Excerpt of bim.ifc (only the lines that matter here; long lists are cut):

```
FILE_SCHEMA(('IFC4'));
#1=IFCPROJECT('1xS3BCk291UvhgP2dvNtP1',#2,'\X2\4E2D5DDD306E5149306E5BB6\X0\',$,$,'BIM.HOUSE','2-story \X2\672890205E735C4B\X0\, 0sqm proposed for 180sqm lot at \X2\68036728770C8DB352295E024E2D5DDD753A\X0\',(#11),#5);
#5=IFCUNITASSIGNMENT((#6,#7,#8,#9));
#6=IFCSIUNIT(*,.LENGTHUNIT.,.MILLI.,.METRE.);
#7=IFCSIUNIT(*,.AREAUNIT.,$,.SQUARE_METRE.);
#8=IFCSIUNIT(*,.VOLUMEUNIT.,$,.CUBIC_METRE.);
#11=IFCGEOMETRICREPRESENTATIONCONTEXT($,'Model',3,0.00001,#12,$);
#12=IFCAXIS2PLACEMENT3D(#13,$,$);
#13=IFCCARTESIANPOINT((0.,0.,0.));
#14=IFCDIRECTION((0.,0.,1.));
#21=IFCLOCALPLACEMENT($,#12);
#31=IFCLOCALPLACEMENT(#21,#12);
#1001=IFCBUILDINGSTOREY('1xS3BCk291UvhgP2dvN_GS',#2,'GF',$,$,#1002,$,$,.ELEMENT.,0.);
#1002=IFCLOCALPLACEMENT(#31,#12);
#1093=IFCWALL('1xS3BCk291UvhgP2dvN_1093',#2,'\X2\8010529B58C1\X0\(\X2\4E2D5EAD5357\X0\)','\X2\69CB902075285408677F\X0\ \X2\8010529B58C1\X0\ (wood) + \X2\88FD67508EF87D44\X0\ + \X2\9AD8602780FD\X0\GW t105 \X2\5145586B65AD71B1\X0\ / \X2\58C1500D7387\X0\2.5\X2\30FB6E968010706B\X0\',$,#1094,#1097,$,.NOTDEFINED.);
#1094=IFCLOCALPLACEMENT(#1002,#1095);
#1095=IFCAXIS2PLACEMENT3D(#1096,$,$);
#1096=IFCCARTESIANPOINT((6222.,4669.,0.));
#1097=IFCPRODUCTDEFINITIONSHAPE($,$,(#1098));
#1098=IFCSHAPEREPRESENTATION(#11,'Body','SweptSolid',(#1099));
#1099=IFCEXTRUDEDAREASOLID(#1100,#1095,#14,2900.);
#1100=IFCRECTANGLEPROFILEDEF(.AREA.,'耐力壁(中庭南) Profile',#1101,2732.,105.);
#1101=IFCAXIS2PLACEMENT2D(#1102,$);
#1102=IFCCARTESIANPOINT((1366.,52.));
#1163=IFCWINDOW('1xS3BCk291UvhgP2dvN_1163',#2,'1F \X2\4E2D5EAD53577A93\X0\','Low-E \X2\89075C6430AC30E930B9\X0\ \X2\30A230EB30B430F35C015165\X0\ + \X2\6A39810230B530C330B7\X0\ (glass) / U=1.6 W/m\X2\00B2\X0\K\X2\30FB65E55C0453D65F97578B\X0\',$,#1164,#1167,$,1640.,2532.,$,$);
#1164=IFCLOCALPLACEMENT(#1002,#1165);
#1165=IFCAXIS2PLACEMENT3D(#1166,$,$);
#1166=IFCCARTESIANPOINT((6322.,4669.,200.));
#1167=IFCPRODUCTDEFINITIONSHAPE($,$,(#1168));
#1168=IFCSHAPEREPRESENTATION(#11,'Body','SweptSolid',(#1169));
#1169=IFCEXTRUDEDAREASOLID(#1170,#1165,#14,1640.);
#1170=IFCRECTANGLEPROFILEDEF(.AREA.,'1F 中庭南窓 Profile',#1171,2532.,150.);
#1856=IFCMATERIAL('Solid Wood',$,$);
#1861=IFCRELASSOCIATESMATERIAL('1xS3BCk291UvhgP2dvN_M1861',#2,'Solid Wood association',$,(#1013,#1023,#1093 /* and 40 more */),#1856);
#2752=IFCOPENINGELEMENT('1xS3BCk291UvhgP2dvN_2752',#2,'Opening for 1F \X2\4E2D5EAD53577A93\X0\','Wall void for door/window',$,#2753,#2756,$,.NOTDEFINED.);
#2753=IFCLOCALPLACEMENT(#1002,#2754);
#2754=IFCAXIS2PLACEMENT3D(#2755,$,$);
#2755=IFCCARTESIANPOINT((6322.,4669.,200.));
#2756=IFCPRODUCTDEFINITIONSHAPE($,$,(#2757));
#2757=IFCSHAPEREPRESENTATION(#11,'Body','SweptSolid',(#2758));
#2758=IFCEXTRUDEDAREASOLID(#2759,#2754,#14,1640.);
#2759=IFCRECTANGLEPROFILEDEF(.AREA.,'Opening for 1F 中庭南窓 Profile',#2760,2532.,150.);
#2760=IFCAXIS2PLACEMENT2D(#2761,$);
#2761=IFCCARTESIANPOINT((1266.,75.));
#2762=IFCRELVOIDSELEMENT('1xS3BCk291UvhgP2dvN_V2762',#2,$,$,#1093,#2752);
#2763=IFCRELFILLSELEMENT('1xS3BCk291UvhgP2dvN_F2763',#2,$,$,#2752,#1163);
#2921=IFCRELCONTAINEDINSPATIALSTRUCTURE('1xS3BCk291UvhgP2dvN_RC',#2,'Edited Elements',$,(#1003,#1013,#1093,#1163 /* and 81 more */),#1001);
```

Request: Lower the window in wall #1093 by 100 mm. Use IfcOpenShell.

```python
import numpy as np
import ifcopenshell
import ifcopenshell.api.geometry
import ifcopenshell.util.placement
import ifcopenshell.util.unit

model = ifcopenshell.open("bim.ifc")
unit_scale = ifcopenshell.util.unit.calculate_unit_scale(model)

window = model.by_guid("1xS3BCk291UvhgP2dvN_1163")
opening = window.FillsVoids[0].RelatingOpeningElement
dz = -0.1 / unit_scale

shift = np.array([0.0, 0.0, dz])
# The window is not placed relative to its opening, so move both.
for product in (opening, window):
    matrix = ifcopenshell.util.placement.get_local_placement(product.ObjectPlacement)
    matrix[:3, 3] += shift
    ifcopenshell.api.geometry.edit_object_placement(model, product=product, matrix=matrix, is_si=False)

print(f"moved by {dz * unit_scale:+.3f} m")

model.write("bim_updated.ifc")
```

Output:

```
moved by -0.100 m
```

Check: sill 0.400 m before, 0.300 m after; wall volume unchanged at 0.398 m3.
